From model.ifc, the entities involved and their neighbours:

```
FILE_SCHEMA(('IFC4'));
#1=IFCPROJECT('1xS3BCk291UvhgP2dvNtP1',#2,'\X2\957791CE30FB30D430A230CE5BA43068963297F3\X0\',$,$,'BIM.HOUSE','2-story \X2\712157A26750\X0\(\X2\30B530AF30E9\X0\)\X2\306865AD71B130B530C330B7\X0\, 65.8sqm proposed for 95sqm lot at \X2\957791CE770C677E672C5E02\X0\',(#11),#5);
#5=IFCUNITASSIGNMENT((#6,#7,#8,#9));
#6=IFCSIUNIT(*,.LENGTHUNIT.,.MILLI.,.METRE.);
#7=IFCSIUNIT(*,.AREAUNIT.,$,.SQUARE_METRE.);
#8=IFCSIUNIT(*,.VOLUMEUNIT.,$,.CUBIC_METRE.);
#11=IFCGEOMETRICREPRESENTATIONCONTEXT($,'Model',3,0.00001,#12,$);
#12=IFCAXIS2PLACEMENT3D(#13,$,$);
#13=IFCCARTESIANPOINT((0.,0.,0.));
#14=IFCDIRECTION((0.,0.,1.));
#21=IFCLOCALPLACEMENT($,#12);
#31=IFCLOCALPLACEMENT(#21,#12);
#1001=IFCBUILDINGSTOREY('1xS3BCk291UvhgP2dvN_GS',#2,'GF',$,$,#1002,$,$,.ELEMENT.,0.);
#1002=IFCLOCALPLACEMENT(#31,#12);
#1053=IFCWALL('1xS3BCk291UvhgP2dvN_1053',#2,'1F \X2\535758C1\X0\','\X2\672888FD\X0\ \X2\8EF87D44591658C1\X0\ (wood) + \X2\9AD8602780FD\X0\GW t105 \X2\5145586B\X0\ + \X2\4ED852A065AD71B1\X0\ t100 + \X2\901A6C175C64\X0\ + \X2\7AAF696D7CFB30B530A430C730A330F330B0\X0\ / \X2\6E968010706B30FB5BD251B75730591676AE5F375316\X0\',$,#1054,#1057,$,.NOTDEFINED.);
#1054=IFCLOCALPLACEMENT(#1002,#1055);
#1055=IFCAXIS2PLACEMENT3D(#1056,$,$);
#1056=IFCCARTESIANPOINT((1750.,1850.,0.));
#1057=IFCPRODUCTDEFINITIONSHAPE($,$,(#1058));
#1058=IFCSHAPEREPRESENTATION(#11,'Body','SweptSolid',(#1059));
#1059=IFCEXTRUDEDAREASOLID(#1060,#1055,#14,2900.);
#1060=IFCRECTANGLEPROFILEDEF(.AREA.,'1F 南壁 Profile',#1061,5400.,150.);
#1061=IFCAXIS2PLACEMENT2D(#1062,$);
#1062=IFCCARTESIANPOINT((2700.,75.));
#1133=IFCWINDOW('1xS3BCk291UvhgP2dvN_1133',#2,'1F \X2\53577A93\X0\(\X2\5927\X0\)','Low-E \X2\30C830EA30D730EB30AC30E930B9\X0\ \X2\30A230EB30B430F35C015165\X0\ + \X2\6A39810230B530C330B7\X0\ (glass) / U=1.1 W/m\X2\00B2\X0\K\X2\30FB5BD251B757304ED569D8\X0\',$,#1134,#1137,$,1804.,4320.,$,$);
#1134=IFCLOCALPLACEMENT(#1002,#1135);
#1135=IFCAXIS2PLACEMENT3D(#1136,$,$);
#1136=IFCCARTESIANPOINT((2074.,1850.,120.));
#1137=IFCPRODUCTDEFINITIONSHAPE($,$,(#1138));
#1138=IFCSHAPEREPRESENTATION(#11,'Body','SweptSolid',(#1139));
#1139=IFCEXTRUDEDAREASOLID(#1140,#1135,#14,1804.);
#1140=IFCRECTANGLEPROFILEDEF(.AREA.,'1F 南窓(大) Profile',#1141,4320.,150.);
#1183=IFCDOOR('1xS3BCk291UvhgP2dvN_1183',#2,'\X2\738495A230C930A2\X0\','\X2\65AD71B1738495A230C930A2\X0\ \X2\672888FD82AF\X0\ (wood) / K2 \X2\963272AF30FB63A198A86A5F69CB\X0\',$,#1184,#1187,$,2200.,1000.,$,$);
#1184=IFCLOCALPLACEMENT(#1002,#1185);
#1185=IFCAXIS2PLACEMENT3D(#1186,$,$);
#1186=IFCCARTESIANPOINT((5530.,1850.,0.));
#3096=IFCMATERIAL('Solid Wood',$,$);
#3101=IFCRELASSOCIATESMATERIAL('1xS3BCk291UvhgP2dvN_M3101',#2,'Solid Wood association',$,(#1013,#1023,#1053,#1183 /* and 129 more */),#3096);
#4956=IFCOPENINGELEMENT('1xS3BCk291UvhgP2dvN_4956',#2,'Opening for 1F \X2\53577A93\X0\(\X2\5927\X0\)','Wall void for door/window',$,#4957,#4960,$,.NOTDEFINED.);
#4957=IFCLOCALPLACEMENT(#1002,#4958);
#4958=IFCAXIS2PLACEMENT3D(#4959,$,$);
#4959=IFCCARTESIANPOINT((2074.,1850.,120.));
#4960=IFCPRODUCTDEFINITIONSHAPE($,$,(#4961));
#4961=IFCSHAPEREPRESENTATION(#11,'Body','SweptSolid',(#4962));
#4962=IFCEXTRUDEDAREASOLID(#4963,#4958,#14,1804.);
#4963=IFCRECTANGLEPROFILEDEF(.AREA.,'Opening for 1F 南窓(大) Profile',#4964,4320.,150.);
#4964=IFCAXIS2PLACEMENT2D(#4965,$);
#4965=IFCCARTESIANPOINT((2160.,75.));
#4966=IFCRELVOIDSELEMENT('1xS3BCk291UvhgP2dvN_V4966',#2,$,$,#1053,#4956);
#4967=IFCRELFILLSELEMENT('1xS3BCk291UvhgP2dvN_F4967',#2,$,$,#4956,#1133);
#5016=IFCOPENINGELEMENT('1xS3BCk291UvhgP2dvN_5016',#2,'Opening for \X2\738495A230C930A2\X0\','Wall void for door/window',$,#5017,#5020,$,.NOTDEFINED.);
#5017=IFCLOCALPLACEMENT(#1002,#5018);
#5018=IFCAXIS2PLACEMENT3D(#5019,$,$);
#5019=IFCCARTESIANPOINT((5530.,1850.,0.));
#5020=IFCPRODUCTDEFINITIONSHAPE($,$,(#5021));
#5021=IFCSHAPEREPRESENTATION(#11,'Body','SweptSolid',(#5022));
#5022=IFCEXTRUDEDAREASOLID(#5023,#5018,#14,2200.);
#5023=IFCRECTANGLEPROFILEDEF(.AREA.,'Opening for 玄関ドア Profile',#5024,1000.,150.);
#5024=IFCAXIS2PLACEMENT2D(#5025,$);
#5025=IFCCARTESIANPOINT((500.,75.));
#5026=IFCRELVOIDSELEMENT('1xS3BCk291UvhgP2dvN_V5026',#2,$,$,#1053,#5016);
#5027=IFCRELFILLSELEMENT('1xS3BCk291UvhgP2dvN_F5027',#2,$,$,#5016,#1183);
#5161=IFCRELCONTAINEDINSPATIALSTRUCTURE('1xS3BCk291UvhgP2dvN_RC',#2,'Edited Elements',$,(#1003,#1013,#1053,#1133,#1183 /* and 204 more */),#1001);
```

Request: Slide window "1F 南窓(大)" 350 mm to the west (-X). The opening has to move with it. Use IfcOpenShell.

```python
import ifcopenshell
import ifcopenshell.api.geometry
import ifcopenshell.util.placement
import ifcopenshell.util.unit

model = ifcopenshell.open("model.ifc")
unit_scale = ifcopenshell.util.unit.calculate_unit_scale(model)

window = model.by_guid("1xS3BCk291UvhgP2dvN_1133")
opening = window.FillsVoids[0].RelatingOpeningElement
wall = opening.VoidsElements[0].RelatingBuildingElement

wall_matrix = ifcopenshell.util.placement.get_local_placement(wall.ObjectPlacement)
shift = wall_matrix[:3, 0] * -0.35 / unit_scale
before = ifcopenshell.util.placement.get_local_placement(window.ObjectPlacement)[:3, 3].copy()

# The window is not placed relative to its opening, so move both.
for product in (opening, window):
    matrix = ifcopenshell.util.placement.get_local_placement(product.ObjectPlacement)
    matrix[:3, 3] += shift
    ifcopenshell.api.geometry.edit_object_placement(model, product=product, matrix=matrix, is_si=False)

after = ifcopenshell.util.placement.get_local_placement(window.ObjectPlacement)[:3, 3]
print("window moved by", (after - before).round(3) + 0.0)

model.write("model_rev.ifc")
```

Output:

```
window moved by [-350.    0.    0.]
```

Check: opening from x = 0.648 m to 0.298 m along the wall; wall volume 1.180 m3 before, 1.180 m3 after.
